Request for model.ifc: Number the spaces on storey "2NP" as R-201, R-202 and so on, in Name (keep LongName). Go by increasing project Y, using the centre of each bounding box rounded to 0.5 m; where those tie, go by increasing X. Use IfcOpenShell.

First a look at what the model holds.

```python
import ifcopenshell
import ifcopenshell.util.element
import ifcopenshell.util.placement

model = ifcopenshell.open("model.ifc")
print(model.schema)
storey = next(s for s in model.by_type("IfcBuildingStorey") if s.Name == "2NP")
spaces = [e for e in ifcopenshell.util.element.get_decomposition(storey) if e.is_a("IfcSpace")]
for e in sorted(spaces, key=lambda e: e.id()):
    origin = ifcopenshell.util.placement.get_local_placement(e.ObjectPlacement)[:3, 3]
    print(e.id(), e.Name, e.LongName, origin.round(2) + 0.0, sep=" | ")
```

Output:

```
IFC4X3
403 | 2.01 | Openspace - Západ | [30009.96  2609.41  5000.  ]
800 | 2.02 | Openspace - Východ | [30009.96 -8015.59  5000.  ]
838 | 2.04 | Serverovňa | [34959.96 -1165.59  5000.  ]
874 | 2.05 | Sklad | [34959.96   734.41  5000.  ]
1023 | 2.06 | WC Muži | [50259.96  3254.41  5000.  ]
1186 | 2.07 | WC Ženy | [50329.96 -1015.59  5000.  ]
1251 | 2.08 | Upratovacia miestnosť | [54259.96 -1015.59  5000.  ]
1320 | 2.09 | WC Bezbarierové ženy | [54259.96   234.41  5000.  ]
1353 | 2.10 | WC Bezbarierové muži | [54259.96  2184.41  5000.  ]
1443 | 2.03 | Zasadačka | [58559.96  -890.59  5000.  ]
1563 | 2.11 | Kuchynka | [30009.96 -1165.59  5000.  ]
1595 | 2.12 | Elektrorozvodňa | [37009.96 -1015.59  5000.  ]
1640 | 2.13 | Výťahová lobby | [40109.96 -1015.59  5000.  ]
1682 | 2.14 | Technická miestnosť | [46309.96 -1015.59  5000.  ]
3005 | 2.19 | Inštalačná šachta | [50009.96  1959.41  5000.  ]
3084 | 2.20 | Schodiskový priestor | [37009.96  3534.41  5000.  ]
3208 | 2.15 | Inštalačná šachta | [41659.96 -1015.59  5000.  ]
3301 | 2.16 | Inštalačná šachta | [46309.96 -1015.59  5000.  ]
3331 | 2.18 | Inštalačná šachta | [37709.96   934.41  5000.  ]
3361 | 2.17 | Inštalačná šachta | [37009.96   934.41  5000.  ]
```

```python
import ifcopenshell
import ifcopenshell.geom
import ifcopenshell.util.element
import ifcopenshell.util.shape

model = ifcopenshell.open("model.ifc")
settings = ifcopenshell.geom.settings()
settings.set("use-world-coords", True)


def centre(element):
    shape = ifcopenshell.geom.create_shape(settings, element)
    return ifcopenshell.util.shape.get_bbox_centroid(shape.geometry)


storey = next(s for s in model.by_type("IfcBuildingStorey") if s.Name == "2NP")
spaces = [e for e in ifcopenshell.util.element.get_decomposition(storey) if e.is_a("IfcSpace")]

# Insertion points can sit at a corner or the storey origin, so sort by the geometry (in metres).
centres = {e: centre(e) for e in spaces}
spaces.sort(key=lambda e: (round(centres[e][1] / 0.5), centres[e][0]))

for i, e in enumerate(spaces, start=1):
    number = f"R-2{i:02d}"
    e.Name = number
    print(e.id(), number)

model.write("model_edited.ifc")
```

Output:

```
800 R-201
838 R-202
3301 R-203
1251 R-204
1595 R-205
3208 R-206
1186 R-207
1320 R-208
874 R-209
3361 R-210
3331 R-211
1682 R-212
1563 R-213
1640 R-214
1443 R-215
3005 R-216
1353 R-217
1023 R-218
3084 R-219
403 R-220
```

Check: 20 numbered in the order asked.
